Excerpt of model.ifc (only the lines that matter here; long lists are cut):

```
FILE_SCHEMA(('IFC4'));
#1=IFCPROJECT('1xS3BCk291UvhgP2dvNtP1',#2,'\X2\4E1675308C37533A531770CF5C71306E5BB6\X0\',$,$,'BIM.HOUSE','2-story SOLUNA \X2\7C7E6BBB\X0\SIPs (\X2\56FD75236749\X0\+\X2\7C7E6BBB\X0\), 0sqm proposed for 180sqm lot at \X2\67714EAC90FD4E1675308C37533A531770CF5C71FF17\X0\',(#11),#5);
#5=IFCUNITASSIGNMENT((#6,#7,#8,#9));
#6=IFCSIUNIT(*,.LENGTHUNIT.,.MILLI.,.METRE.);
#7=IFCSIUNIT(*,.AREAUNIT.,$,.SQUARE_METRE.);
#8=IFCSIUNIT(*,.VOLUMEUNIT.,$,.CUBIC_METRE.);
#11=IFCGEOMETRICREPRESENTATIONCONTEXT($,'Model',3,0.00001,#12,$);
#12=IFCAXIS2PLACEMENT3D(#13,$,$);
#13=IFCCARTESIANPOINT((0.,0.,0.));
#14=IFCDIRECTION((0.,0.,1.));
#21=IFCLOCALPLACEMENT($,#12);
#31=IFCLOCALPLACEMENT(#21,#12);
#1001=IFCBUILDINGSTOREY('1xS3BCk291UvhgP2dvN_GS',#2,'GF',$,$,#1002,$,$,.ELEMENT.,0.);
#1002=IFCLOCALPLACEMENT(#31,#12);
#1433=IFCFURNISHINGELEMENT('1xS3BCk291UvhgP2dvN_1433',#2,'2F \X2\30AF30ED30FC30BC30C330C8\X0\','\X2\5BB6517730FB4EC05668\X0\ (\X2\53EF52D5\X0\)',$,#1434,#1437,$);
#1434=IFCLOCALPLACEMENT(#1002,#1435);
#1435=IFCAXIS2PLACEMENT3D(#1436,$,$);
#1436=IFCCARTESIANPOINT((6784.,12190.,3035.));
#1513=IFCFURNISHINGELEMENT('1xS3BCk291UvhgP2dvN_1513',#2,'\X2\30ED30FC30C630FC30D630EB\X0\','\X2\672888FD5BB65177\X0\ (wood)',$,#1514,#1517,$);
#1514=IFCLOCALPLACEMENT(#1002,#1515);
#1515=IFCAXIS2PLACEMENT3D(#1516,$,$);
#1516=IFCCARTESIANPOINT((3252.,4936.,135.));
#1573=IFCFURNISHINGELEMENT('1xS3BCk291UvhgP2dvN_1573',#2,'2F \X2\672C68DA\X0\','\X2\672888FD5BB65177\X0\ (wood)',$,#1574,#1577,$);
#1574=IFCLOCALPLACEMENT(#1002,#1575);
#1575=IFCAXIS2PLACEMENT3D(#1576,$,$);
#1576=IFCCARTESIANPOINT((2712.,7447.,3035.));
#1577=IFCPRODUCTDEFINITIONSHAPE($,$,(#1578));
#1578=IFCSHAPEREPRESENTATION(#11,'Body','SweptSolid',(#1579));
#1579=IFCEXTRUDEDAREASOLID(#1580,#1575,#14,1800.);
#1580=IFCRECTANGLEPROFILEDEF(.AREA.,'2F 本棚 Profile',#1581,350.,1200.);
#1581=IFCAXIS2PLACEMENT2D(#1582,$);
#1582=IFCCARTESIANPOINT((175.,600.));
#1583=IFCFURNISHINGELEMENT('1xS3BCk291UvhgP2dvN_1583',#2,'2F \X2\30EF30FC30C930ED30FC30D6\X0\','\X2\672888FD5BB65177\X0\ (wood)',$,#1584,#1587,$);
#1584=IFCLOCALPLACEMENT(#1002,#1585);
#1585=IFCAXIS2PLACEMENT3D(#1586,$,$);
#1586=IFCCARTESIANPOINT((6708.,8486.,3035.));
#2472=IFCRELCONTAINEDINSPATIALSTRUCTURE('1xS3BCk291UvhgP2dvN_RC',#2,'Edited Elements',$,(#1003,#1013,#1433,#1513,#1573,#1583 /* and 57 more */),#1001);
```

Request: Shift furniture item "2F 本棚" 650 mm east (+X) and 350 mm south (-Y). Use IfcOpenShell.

```python
import ifcopenshell
import ifcopenshell.api.geometry
import ifcopenshell.util.placement
import ifcopenshell.util.unit

model = ifcopenshell.open("model.ifc")
unit_scale = ifcopenshell.util.unit.calculate_unit_scale(model)

item = model.by_id(1573)
matrix = ifcopenshell.util.placement.get_local_placement(item.ObjectPlacement)
matrix[0, 3] += 0.65 / unit_scale
matrix[1, 3] -= 0.35 / unit_scale
ifcopenshell.api.geometry.edit_object_placement(model, product=item, matrix=matrix, is_si=False)

print(ifcopenshell.util.placement.get_local_placement(item.ObjectPlacement).round(3) + 0.0)

model.write("model_rev.ifc")
```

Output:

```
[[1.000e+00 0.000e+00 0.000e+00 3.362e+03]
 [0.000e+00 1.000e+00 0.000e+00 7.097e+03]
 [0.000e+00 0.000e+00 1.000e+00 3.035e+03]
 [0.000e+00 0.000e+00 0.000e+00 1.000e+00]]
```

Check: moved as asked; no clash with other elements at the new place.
